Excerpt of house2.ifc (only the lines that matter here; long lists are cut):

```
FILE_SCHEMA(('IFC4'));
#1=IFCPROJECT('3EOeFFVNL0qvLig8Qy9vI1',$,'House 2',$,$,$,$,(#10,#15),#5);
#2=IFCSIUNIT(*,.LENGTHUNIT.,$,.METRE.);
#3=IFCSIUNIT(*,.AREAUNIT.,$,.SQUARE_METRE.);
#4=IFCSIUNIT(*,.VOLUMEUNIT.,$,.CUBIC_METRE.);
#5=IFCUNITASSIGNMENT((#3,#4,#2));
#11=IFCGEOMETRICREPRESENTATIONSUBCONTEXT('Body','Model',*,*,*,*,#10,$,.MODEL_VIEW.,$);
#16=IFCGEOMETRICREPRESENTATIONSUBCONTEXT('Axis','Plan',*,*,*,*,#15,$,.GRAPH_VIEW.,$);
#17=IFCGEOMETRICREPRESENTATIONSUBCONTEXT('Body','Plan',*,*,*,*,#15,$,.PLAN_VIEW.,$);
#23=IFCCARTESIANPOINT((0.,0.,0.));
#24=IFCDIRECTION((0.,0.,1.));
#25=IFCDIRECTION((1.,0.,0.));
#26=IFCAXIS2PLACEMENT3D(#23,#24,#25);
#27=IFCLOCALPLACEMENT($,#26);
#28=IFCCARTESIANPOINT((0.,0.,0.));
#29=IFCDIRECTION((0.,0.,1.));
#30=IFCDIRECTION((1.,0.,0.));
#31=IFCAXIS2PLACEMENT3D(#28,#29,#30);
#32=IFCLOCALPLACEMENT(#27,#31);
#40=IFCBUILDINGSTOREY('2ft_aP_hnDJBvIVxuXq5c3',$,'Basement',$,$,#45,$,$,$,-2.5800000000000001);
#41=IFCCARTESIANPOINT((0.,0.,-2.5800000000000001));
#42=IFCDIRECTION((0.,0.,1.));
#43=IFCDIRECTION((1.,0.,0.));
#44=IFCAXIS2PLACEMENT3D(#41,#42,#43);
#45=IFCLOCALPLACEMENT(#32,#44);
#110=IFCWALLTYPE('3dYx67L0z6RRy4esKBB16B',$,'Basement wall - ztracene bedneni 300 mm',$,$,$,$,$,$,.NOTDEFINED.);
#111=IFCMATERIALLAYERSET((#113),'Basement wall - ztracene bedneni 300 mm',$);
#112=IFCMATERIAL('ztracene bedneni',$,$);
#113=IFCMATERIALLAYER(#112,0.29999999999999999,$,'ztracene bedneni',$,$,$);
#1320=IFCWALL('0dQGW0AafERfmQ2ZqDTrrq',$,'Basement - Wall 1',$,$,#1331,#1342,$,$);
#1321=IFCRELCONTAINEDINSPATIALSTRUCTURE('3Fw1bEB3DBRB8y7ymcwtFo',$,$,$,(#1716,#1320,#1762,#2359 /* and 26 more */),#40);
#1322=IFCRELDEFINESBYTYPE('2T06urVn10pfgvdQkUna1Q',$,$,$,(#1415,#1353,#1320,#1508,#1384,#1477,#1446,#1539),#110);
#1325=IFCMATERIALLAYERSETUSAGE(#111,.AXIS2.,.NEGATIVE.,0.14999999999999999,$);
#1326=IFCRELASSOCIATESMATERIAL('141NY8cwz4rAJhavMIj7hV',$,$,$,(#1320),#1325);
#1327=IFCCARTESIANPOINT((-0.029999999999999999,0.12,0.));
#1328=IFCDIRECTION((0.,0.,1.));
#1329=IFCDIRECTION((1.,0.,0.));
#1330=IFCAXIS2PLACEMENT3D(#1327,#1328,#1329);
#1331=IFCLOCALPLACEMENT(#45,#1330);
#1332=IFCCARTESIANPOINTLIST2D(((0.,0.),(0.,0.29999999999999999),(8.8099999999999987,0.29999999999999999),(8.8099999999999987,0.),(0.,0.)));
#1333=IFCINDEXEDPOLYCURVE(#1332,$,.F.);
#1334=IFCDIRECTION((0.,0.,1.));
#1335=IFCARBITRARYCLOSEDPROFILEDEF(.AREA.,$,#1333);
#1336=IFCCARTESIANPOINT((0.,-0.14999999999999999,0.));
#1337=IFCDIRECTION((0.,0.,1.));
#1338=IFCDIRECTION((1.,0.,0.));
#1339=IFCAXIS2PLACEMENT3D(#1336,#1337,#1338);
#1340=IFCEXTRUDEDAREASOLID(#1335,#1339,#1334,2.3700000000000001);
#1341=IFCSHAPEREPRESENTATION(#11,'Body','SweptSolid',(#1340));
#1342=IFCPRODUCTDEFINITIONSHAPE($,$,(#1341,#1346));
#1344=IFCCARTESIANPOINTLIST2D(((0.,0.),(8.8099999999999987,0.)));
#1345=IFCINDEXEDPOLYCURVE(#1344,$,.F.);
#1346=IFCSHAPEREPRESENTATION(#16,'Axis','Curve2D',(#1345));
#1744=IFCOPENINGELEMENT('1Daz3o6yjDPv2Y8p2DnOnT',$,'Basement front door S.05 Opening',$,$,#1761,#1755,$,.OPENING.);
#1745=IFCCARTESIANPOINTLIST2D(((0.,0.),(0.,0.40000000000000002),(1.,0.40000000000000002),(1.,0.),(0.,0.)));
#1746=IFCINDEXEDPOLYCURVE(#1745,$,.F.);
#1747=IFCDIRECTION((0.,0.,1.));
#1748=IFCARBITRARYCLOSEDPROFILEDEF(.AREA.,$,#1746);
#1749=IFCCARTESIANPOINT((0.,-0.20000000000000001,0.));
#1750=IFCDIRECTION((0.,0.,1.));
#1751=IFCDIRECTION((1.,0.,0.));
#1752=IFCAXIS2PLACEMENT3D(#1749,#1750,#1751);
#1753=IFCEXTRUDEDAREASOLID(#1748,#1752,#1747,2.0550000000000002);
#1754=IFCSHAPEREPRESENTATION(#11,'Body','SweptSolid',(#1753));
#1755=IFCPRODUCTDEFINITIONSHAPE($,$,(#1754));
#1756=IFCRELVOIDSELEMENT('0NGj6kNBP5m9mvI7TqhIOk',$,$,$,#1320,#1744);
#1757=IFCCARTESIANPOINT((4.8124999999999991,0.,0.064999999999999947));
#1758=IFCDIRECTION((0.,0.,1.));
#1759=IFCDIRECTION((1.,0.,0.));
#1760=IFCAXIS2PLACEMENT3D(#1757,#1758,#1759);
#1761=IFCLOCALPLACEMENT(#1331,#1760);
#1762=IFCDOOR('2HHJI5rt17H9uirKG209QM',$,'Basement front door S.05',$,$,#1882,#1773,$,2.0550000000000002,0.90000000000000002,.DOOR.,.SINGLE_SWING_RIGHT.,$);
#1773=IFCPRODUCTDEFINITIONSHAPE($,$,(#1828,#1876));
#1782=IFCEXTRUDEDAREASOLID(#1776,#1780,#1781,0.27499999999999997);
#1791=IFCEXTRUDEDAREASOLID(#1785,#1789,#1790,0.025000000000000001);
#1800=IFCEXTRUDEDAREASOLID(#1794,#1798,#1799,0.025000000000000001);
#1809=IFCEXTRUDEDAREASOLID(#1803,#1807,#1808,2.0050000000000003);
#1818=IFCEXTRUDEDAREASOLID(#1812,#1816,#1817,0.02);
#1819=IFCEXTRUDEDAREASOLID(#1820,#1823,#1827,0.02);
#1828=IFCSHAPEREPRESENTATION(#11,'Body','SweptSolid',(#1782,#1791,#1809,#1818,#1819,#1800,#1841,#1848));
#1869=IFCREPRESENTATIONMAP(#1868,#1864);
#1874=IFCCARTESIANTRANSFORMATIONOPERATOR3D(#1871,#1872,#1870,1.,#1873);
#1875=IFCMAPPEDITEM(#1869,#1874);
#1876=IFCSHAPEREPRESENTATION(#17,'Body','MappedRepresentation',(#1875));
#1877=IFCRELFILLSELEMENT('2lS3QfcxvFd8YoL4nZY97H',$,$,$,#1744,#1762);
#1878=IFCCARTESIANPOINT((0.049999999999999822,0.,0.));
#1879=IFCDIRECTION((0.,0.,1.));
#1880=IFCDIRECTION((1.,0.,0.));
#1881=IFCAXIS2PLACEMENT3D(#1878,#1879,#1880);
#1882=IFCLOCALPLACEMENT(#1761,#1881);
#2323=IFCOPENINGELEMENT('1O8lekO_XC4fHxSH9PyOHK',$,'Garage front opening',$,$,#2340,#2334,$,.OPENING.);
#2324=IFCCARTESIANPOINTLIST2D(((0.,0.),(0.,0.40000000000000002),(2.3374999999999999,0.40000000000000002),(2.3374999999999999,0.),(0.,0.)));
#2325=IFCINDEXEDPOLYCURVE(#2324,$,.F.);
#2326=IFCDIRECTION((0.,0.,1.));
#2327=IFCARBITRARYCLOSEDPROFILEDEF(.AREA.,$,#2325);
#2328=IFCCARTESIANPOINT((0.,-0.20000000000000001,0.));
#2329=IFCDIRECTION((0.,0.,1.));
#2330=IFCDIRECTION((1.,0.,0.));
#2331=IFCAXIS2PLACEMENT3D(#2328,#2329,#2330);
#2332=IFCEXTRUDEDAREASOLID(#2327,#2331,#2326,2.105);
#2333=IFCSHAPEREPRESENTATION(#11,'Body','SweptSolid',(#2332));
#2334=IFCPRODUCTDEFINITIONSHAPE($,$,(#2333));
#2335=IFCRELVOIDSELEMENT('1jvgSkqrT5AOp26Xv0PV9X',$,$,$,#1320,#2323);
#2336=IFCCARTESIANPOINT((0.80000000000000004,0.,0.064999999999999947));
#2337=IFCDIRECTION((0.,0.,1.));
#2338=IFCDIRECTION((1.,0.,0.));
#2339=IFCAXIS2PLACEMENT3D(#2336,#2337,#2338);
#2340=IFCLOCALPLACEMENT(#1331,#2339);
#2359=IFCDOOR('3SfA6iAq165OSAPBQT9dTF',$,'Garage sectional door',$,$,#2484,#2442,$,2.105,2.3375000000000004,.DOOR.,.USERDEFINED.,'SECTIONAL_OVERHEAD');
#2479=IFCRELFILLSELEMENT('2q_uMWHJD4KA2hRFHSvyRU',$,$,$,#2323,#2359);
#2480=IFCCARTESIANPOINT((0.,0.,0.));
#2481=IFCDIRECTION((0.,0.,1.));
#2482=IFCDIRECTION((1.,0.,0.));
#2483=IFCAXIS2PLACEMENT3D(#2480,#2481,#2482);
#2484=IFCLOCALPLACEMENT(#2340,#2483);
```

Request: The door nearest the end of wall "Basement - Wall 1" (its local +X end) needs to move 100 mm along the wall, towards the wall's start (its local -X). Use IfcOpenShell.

```python
import ifcopenshell
import ifcopenshell.api.geometry
import ifcopenshell.util.placement

model = ifcopenshell.open("house2.ifc")

door = model.by_guid("2HHJI5rt17H9uirKG209QM")
opening = door.FillsVoids[0].RelatingOpeningElement
wall = opening.VoidsElements[0].RelatingBuildingElement

wall_matrix = ifcopenshell.util.placement.get_local_placement(wall.ObjectPlacement)
shift = wall_matrix[:3, 0] * -0.1
before = ifcopenshell.util.placement.get_local_placement(door.ObjectPlacement)[:3, 3].copy()

# The door is placed relative to its opening, so it follows when the opening moves.
matrix = ifcopenshell.util.placement.get_local_placement(opening.ObjectPlacement)
matrix[:3, 3] += shift
ifcopenshell.api.geometry.edit_object_placement(
    model, product=opening, matrix=matrix, is_si=False, should_transform_children=True
)

after = ifcopenshell.util.placement.get_local_placement(door.ObjectPlacement)[:3, 3]
print("door moved by", (after - before).round(3) + 0.0)

model.write("house2_updated.ifc")
```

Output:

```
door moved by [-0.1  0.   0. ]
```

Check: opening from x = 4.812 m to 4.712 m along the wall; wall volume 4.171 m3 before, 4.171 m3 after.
